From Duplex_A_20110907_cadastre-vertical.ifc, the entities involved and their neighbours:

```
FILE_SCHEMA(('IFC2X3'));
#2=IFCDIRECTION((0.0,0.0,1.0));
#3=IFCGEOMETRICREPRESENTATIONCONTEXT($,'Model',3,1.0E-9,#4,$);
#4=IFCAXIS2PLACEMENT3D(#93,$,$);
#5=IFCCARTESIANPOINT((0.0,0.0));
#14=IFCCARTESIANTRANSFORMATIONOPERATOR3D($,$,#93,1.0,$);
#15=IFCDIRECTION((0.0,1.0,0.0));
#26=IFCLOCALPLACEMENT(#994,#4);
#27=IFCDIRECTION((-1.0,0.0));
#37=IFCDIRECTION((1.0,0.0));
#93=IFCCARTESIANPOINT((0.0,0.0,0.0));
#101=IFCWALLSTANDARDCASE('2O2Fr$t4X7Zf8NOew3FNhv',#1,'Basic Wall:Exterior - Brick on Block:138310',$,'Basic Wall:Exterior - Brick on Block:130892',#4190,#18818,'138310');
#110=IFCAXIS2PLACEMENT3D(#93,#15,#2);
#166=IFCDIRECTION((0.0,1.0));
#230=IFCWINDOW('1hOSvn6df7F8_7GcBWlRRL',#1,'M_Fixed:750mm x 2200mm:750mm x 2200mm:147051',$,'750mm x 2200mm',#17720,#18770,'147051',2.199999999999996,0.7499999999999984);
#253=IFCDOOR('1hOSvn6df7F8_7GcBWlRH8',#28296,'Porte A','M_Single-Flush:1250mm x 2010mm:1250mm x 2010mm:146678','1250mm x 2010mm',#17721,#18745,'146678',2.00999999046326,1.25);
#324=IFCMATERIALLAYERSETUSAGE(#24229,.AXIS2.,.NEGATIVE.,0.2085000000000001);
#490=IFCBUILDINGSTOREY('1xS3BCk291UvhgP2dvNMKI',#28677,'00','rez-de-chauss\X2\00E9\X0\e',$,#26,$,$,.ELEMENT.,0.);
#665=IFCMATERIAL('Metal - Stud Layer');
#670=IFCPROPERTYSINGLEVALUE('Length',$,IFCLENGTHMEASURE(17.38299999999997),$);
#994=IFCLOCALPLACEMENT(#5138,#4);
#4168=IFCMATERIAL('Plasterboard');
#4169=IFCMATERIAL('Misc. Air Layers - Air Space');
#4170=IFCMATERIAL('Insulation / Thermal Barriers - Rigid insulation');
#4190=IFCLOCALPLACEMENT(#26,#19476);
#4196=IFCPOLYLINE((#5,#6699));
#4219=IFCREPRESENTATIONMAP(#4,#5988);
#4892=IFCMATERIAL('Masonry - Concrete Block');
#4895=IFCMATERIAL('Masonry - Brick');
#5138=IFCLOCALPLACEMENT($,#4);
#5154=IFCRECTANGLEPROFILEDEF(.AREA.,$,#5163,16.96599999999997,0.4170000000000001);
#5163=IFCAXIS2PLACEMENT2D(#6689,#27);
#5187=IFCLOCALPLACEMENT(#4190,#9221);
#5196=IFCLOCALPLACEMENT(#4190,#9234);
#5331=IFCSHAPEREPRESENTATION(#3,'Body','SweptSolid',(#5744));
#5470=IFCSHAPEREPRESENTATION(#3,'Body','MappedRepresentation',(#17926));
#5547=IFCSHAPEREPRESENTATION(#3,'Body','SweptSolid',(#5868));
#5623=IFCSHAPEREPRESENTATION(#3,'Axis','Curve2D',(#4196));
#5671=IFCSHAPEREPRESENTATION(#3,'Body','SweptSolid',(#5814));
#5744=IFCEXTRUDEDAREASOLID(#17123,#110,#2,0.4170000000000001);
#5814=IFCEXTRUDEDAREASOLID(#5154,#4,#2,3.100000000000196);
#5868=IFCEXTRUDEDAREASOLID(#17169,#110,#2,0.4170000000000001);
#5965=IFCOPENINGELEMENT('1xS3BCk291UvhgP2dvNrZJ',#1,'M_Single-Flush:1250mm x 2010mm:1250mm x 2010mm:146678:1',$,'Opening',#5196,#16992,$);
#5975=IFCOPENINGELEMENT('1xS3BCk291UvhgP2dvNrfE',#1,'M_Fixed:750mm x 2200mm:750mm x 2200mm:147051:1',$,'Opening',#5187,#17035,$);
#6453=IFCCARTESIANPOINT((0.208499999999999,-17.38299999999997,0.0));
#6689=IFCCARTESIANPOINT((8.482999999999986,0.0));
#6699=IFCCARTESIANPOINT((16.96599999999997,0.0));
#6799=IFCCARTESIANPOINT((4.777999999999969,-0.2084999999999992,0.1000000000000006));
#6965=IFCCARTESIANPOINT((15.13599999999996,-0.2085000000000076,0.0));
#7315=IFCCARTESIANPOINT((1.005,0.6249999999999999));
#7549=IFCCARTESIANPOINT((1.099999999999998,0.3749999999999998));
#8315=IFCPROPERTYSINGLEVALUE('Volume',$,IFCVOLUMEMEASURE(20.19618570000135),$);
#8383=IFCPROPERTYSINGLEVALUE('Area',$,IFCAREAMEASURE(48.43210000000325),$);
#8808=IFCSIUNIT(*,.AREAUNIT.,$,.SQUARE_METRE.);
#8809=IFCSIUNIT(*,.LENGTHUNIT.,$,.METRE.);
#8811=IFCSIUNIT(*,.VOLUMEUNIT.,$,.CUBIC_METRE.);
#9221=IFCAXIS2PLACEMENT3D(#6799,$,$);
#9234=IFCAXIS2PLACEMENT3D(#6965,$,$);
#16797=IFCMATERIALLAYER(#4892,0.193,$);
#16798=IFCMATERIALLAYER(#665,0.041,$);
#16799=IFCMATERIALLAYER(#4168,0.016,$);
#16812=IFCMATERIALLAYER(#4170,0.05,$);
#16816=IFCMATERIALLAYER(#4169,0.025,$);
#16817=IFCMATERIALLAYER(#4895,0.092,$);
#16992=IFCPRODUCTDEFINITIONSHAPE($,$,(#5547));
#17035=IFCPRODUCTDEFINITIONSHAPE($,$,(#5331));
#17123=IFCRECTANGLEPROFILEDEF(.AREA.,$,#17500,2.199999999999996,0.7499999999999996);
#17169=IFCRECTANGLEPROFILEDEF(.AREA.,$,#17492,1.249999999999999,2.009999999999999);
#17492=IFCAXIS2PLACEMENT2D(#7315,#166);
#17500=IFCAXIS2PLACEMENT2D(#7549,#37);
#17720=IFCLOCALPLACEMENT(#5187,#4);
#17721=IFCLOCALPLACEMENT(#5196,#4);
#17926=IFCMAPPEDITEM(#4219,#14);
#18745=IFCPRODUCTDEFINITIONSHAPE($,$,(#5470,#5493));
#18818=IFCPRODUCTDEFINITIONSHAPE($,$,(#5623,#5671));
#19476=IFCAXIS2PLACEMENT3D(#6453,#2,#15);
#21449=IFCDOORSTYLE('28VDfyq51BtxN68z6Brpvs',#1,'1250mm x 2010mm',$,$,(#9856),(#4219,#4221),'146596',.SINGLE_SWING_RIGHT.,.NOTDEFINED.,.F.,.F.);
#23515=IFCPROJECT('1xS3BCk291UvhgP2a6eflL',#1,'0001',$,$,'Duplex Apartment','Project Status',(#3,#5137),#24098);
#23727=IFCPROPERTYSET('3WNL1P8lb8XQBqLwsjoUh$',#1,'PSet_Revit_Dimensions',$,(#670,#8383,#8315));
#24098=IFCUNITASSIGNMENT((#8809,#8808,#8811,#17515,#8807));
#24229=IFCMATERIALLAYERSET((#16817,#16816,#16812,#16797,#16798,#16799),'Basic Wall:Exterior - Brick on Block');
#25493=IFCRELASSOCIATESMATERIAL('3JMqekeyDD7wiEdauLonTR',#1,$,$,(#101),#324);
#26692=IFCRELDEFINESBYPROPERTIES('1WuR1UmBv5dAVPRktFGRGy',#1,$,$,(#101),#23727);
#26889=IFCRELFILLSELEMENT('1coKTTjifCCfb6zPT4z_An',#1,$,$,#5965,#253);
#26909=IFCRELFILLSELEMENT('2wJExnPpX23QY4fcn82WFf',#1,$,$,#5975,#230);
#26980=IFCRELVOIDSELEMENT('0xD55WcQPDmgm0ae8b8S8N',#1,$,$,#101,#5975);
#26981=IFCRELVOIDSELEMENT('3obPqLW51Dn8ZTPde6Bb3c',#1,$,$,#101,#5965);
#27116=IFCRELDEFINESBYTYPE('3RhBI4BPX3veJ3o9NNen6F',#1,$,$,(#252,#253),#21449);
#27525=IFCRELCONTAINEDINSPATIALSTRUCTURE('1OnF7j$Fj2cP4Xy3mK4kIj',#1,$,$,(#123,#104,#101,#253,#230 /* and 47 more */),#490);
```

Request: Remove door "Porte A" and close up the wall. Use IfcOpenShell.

```python
import ifcopenshell
import ifcopenshell.api.feature
import ifcopenshell.api.pset
import ifcopenshell.api.root
import ifcopenshell.geom
import ifcopenshell.util.element
import ifcopenshell.util.shape
import ifcopenshell.util.unit

model = ifcopenshell.open("Duplex_A_20110907_cadastre-vertical.ifc")
area_scale = ifcopenshell.util.unit.calculate_unit_scale(model, "AREAUNIT")
volume_scale = ifcopenshell.util.unit.calculate_unit_scale(model, "VOLUMEUNIT")
settings = ifcopenshell.geom.settings()


def volume(element):
    """Net volume in cubic metres, openings subtracted."""
    shape = ifcopenshell.geom.create_shape(settings, element)
    return ifcopenshell.util.shape.get_volume(shape.geometry)


door = model.by_guid("1hOSvn6df7F8_7GcBWlRH8")
opening = door.FillsVoids[0].RelatingOpeningElement
wall = opening.VoidsElements[0].RelatingBuildingElement
before = volume(wall)

ifcopenshell.api.root.remove_product(model, product=door)
ifcopenshell.api.feature.remove_feature(model, feature=opening)

after = volume(wall)
thickness = 0.417  # wall thickness in metres

# Update the wall's stored quantities.
pset = model.by_id(ifcopenshell.util.element.get_pset(wall, "PSet_Revit_Dimensions", should_inherit=False)["id"])
ifcopenshell.api.pset.edit_pset(model, pset=pset, properties={
    "Area": model.create_entity("IfcAreaMeasure", after / thickness / area_scale),
    "Volume": model.create_entity("IfcVolumeMeasure", after / volume_scale),
})

print(f"wall volume {before:.3f} -> {after:.3f} m3")

model.write("Duplex_A_20110907_cadastre-vertical_edited.ifc")
```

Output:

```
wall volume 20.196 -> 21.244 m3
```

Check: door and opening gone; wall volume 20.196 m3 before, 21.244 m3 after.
